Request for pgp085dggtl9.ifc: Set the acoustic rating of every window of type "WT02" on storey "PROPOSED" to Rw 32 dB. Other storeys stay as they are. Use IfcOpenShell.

First a look at what the model holds.

```python
import ifcopenshell
import ifcopenshell.util.element

model = ifcopenshell.open("pgp085dggtl9.ifc")
print(model.schema)
storey = next(s for s in model.by_type("IfcBuildingStorey") if s.Name == "PROPOSED")
windows = [e for e in ifcopenshell.util.element.get_decomposition(storey) if e.is_a("IfcWindow")]
seen = {}
for e in windows:
    element_type = ifcopenshell.util.element.get_type(e)
    key = (element_type.Name if element_type != e and element_type else None, ifcopenshell.util.element.get_pset(e, "Pset_WindowCommon", "AcousticRating"))
    seen[key] = seen.get(key, 0) + 1
for (name, value), count in sorted(seen.items(), key=str):
    print(count, "x", name, "|", value)
```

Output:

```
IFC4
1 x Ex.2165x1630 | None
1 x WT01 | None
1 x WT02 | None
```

```python
import ifcopenshell
import ifcopenshell.api.pset
import ifcopenshell.util.element

model = ifcopenshell.open("pgp085dggtl9.ifc")

storey = next(s for s in model.by_type("IfcBuildingStorey") if s.Name == "PROPOSED")
windows = [e for e in ifcopenshell.util.element.get_decomposition(storey) if e.is_a("IfcWindow")]

count = 0
for e in windows:
    element_type = ifcopenshell.util.element.get_type(e)
    if element_type in (None, e) or element_type.Name != "WT02":
        continue
    # add_pset returns the element's existing set when there is one.
    pset = ifcopenshell.api.pset.add_pset(model, product=e, name="Pset_WindowCommon")
    ifcopenshell.api.pset.edit_pset(model, pset=pset, properties={"AcousticRating": "Rw 32 dB"})
    count += 1

print(count, "windows updated")

model.write("pgp085dggtl9_edited.ifc")
```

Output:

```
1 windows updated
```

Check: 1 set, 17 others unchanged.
